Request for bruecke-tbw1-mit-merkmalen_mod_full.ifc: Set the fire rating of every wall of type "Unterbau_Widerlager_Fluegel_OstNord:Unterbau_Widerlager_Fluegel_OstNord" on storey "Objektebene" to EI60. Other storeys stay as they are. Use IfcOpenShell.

First a look at what the model holds.

```python
import ifcopenshell
import ifcopenshell.util.element

model = ifcopenshell.open("bruecke-tbw1-mit-merkmalen_mod_full.ifc")
print(model.schema)
storey = next(s for s in model.by_type("IfcBuildingStorey") if s.Name == "Objektebene")
walls = [e for e in ifcopenshell.util.element.get_decomposition(storey) if e.is_a("IfcWall")]
seen = {}
for e in walls:
    element_type = ifcopenshell.util.element.get_type(e)
    key = (element_type.Name if element_type != e and element_type else None, ifcopenshell.util.element.get_pset(e, "Pset_WallCommon", "FireRating"))
    seen[key] = seen.get(key, 0) + 1
for (name, value), count in sorted(seen.items(), key=str):
    print(count, "x", name, "|", value)
```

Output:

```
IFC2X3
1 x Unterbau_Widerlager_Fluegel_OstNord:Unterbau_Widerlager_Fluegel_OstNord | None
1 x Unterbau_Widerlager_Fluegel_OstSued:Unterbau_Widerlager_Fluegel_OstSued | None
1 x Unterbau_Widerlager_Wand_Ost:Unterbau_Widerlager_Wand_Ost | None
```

```python
import ifcopenshell
import ifcopenshell.api.pset
import ifcopenshell.util.element

model = ifcopenshell.open("bruecke-tbw1-mit-merkmalen_mod_full.ifc")

storey = next(s for s in model.by_type("IfcBuildingStorey") if s.Name == "Objektebene")
walls = [e for e in ifcopenshell.util.element.get_decomposition(storey) if e.is_a("IfcWall")]

count = 0
for e in walls:
    element_type = ifcopenshell.util.element.get_type(e)
    if element_type in (None, e) or element_type.Name != "Unterbau_Widerlager_Fluegel_OstNord:Unterbau_Widerlager_Fluegel_OstNord":
        continue
    # add_pset returns the element's existing set when there is one.
    pset = ifcopenshell.api.pset.add_pset(model, product=e, name="Pset_WallCommon")
    ifcopenshell.api.pset.edit_pset(model, pset=pset, properties={"FireRating": "EI60"})
    count += 1

print(count, "walls updated")

model.write("bruecke-tbw1-mit-merkmalen_mod_full_edited.ifc")
```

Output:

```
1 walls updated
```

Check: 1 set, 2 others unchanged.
